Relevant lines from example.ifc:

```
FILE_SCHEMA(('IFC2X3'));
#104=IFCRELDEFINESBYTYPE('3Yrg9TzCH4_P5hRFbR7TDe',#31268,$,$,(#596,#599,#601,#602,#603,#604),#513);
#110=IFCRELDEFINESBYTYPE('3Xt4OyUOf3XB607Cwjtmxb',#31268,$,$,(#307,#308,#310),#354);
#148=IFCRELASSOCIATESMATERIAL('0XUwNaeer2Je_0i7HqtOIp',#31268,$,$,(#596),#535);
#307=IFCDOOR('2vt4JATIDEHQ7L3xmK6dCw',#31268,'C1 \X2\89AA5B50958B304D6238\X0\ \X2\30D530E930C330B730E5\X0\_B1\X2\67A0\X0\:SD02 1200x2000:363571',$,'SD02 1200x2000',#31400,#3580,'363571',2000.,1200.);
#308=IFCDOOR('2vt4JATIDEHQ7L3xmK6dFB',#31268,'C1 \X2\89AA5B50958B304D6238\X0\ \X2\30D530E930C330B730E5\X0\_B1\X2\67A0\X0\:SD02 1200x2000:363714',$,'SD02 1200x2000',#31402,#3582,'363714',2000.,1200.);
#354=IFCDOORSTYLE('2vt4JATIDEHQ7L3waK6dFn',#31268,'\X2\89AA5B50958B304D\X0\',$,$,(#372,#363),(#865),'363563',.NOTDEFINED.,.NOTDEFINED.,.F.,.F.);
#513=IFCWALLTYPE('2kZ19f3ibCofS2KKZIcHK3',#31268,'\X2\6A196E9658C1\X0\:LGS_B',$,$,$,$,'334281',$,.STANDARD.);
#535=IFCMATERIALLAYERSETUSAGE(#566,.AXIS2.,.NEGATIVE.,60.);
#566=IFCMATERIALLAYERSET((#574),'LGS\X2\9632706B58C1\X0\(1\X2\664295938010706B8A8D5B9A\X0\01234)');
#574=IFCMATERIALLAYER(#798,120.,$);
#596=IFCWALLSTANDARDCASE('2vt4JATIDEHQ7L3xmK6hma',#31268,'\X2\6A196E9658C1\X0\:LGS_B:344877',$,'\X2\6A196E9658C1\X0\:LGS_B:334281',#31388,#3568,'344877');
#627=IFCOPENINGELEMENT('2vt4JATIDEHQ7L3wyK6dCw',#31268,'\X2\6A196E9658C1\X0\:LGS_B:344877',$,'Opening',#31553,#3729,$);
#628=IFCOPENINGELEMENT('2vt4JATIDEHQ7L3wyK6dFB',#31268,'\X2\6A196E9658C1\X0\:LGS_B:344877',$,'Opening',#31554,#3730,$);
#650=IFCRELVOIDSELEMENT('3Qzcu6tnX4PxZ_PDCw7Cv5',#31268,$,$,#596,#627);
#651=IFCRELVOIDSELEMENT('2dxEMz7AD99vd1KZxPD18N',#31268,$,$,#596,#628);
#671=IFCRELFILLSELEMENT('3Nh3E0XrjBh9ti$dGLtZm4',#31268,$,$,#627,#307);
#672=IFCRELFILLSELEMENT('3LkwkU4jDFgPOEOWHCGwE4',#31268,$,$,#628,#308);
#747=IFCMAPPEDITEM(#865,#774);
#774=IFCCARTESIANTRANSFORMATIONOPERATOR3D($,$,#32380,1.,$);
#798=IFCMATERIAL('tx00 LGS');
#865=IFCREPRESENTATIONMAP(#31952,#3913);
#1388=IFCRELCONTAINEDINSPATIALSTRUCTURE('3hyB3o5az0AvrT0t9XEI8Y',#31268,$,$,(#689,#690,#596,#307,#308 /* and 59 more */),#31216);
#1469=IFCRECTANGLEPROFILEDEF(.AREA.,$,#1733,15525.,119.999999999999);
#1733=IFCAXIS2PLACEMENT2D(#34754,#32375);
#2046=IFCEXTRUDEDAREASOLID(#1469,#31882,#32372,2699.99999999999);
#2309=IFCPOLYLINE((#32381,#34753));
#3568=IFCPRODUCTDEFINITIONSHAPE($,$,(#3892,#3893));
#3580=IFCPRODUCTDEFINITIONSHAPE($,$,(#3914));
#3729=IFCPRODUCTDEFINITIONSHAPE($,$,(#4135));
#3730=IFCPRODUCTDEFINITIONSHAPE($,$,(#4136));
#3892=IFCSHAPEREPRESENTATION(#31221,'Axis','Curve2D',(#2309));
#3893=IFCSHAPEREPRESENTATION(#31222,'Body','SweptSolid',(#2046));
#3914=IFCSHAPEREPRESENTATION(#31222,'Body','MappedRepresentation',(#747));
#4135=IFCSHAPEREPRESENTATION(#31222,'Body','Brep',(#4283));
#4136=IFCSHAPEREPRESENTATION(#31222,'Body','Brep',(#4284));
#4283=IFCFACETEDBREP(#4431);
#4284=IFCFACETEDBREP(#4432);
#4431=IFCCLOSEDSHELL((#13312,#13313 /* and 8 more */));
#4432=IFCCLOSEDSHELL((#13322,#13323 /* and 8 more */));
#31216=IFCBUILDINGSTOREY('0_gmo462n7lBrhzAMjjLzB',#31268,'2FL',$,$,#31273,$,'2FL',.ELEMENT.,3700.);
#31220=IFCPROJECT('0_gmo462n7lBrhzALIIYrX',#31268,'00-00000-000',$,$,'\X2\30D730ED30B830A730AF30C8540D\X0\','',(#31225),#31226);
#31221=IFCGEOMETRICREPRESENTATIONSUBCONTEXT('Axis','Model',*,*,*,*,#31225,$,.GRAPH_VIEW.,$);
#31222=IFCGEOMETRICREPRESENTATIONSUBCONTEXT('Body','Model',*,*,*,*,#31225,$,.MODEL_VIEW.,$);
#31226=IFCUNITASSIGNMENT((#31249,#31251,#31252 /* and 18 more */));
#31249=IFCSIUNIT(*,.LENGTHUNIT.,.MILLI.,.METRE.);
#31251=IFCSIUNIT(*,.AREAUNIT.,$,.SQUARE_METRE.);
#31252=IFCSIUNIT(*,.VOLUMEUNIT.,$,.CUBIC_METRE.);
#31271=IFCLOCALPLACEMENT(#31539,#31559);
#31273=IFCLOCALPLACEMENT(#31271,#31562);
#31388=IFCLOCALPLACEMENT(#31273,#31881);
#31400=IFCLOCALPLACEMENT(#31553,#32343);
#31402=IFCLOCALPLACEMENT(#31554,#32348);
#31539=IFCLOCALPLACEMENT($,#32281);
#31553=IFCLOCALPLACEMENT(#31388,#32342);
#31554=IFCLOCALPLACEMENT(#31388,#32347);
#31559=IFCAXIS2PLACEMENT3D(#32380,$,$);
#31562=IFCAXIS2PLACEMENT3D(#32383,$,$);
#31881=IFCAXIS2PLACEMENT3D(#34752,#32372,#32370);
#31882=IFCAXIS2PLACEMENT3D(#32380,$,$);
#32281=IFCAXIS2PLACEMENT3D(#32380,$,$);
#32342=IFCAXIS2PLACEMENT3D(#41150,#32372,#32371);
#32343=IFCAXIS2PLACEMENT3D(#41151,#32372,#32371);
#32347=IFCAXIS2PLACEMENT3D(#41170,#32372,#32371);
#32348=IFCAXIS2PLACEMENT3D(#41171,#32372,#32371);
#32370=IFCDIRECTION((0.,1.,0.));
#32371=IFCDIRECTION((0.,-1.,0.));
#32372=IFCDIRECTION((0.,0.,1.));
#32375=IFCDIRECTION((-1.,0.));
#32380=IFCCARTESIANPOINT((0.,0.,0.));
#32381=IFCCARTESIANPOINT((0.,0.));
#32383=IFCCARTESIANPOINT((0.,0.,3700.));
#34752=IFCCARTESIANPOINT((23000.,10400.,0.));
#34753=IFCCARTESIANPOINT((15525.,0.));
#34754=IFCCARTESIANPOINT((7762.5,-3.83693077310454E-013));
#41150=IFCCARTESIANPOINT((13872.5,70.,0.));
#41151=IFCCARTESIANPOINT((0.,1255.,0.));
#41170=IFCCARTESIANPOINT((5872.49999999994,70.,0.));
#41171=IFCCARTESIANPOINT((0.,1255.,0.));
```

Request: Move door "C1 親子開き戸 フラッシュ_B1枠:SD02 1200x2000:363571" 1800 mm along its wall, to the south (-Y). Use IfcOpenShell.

```python
import ifcopenshell
import ifcopenshell.api.geometry
import ifcopenshell.util.placement

model = ifcopenshell.open("example.ifc")

door = model.by_guid("2vt4JATIDEHQ7L3xmK6dCw")
opening = door.FillsVoids[0].RelatingOpeningElement
wall = opening.VoidsElements[0].RelatingBuildingElement

wall_matrix = ifcopenshell.util.placement.get_local_placement(wall.ObjectPlacement)
shift = wall_matrix[:3, 0] * -1800.0
before = ifcopenshell.util.placement.get_local_placement(door.ObjectPlacement)[:3, 3].copy()

# The door is placed relative to its opening, so it follows when the opening moves.
matrix = ifcopenshell.util.placement.get_local_placement(opening.ObjectPlacement)
matrix[:3, 3] += shift
ifcopenshell.api.geometry.edit_object_placement(
    model, product=opening, matrix=matrix, is_si=False, should_transform_children=True
)

after = ifcopenshell.util.placement.get_local_placement(door.ObjectPlacement)[:3, 3]
print("door moved by", (after - before).round(3) + 0.0)

model.write("example_edited.ifc")
```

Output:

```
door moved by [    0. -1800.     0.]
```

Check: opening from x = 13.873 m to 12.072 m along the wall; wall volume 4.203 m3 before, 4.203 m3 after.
